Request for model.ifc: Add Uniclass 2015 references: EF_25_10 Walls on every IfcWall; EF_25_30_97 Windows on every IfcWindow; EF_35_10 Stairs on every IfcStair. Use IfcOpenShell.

First a look at what the model holds.

```python
import ifcopenshell

model = ifcopenshell.open("model.ifc")
print(model.schema)
print("classifications:", [c.Name for c in model.by_type("IfcClassification")])
for ifc_class in ("IfcDoor", "IfcRoof", "IfcStair", "IfcWall", "IfcWindow"):
    print(ifc_class, len(model.by_type(ifc_class)))
```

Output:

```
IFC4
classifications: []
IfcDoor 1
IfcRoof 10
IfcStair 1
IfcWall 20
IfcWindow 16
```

```python
import ifcopenshell
import ifcopenshell.api.classification

model = ifcopenshell.open("model.ifc")

system = ifcopenshell.api.classification.add_classification(model, classification="Uniclass 2015")

codes = {
    "IfcWall": ("EF_25_10", "Walls"),
    "IfcWindow": ("EF_25_30_97", "Windows"),
    "IfcStair": ("EF_35_10", "Stairs"),
}
for ifc_class, (code, name) in codes.items():
    products = model.by_type(ifc_class)
    ifcopenshell.api.classification.add_reference(
        model, products=products, classification=system, identification=code, name=name
    )
    print(code, len(products))

model.write("model_v2.ifc")
```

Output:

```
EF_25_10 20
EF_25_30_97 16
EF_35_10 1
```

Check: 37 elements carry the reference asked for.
